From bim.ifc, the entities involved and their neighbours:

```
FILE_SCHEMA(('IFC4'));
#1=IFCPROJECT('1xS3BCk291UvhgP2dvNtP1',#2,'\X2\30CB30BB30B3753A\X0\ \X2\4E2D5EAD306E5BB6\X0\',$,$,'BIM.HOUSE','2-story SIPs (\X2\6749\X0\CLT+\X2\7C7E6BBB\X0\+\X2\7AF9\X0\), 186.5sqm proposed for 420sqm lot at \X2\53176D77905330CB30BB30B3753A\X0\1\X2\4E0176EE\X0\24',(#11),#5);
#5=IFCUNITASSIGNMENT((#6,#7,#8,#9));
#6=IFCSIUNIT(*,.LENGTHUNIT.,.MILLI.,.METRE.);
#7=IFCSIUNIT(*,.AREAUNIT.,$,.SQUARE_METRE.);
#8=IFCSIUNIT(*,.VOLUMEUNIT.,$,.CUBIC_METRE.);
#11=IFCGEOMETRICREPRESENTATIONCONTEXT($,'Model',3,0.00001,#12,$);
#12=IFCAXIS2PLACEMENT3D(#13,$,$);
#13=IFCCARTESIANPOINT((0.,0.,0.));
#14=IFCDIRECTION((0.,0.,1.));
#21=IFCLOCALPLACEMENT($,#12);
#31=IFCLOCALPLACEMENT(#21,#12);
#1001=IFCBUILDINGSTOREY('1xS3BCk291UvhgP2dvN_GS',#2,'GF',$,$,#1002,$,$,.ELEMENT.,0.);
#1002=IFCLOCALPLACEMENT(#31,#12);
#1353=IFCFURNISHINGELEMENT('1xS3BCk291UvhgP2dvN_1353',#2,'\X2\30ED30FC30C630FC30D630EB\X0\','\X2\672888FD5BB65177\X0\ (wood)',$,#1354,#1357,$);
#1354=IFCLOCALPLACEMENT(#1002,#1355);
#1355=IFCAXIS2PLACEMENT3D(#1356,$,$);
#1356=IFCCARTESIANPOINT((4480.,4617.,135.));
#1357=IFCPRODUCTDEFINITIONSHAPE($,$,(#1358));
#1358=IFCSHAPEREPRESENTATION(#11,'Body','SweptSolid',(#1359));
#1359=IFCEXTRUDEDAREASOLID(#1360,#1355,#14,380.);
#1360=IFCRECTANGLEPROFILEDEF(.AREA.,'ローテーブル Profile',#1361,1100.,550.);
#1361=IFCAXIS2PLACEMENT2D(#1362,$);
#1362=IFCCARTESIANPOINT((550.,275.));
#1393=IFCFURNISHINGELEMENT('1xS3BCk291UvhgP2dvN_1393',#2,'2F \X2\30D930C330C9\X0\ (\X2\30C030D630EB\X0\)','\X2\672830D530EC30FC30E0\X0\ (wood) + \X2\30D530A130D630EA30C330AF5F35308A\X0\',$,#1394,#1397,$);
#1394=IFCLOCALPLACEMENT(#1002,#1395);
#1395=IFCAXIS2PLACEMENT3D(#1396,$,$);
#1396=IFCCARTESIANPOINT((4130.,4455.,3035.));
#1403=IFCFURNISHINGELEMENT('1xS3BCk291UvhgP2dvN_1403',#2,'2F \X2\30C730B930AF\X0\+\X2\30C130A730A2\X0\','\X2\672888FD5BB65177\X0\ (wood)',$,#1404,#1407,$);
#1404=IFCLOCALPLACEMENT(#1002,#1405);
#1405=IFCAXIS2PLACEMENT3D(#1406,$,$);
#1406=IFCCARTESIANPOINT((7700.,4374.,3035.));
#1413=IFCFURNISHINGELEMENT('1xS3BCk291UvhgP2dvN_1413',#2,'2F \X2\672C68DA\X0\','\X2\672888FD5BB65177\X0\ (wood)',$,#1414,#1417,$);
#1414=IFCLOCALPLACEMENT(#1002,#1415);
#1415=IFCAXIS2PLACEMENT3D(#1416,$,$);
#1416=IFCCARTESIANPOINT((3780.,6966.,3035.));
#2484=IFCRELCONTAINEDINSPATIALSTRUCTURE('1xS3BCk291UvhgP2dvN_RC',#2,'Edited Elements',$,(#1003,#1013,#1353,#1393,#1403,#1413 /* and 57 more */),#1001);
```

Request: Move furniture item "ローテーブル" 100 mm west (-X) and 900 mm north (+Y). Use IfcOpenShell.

```python
import ifcopenshell
import ifcopenshell.api.geometry
import ifcopenshell.util.placement

model = ifcopenshell.open("bim.ifc")

item = model.by_guid("1xS3BCk291UvhgP2dvN_1353")
matrix = ifcopenshell.util.placement.get_local_placement(item.ObjectPlacement)
matrix[0, 3] -= 100.0
matrix[1, 3] += 900.0
ifcopenshell.api.geometry.edit_object_placement(model, product=item, matrix=matrix, is_si=False)

print(ifcopenshell.util.placement.get_local_placement(item.ObjectPlacement).round(3) + 0.0)

model.write("bim_updated.ifc")
```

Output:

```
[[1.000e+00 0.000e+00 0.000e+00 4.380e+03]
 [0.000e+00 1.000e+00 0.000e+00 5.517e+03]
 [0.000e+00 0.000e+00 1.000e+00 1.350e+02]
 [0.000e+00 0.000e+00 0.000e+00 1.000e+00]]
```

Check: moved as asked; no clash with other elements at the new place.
